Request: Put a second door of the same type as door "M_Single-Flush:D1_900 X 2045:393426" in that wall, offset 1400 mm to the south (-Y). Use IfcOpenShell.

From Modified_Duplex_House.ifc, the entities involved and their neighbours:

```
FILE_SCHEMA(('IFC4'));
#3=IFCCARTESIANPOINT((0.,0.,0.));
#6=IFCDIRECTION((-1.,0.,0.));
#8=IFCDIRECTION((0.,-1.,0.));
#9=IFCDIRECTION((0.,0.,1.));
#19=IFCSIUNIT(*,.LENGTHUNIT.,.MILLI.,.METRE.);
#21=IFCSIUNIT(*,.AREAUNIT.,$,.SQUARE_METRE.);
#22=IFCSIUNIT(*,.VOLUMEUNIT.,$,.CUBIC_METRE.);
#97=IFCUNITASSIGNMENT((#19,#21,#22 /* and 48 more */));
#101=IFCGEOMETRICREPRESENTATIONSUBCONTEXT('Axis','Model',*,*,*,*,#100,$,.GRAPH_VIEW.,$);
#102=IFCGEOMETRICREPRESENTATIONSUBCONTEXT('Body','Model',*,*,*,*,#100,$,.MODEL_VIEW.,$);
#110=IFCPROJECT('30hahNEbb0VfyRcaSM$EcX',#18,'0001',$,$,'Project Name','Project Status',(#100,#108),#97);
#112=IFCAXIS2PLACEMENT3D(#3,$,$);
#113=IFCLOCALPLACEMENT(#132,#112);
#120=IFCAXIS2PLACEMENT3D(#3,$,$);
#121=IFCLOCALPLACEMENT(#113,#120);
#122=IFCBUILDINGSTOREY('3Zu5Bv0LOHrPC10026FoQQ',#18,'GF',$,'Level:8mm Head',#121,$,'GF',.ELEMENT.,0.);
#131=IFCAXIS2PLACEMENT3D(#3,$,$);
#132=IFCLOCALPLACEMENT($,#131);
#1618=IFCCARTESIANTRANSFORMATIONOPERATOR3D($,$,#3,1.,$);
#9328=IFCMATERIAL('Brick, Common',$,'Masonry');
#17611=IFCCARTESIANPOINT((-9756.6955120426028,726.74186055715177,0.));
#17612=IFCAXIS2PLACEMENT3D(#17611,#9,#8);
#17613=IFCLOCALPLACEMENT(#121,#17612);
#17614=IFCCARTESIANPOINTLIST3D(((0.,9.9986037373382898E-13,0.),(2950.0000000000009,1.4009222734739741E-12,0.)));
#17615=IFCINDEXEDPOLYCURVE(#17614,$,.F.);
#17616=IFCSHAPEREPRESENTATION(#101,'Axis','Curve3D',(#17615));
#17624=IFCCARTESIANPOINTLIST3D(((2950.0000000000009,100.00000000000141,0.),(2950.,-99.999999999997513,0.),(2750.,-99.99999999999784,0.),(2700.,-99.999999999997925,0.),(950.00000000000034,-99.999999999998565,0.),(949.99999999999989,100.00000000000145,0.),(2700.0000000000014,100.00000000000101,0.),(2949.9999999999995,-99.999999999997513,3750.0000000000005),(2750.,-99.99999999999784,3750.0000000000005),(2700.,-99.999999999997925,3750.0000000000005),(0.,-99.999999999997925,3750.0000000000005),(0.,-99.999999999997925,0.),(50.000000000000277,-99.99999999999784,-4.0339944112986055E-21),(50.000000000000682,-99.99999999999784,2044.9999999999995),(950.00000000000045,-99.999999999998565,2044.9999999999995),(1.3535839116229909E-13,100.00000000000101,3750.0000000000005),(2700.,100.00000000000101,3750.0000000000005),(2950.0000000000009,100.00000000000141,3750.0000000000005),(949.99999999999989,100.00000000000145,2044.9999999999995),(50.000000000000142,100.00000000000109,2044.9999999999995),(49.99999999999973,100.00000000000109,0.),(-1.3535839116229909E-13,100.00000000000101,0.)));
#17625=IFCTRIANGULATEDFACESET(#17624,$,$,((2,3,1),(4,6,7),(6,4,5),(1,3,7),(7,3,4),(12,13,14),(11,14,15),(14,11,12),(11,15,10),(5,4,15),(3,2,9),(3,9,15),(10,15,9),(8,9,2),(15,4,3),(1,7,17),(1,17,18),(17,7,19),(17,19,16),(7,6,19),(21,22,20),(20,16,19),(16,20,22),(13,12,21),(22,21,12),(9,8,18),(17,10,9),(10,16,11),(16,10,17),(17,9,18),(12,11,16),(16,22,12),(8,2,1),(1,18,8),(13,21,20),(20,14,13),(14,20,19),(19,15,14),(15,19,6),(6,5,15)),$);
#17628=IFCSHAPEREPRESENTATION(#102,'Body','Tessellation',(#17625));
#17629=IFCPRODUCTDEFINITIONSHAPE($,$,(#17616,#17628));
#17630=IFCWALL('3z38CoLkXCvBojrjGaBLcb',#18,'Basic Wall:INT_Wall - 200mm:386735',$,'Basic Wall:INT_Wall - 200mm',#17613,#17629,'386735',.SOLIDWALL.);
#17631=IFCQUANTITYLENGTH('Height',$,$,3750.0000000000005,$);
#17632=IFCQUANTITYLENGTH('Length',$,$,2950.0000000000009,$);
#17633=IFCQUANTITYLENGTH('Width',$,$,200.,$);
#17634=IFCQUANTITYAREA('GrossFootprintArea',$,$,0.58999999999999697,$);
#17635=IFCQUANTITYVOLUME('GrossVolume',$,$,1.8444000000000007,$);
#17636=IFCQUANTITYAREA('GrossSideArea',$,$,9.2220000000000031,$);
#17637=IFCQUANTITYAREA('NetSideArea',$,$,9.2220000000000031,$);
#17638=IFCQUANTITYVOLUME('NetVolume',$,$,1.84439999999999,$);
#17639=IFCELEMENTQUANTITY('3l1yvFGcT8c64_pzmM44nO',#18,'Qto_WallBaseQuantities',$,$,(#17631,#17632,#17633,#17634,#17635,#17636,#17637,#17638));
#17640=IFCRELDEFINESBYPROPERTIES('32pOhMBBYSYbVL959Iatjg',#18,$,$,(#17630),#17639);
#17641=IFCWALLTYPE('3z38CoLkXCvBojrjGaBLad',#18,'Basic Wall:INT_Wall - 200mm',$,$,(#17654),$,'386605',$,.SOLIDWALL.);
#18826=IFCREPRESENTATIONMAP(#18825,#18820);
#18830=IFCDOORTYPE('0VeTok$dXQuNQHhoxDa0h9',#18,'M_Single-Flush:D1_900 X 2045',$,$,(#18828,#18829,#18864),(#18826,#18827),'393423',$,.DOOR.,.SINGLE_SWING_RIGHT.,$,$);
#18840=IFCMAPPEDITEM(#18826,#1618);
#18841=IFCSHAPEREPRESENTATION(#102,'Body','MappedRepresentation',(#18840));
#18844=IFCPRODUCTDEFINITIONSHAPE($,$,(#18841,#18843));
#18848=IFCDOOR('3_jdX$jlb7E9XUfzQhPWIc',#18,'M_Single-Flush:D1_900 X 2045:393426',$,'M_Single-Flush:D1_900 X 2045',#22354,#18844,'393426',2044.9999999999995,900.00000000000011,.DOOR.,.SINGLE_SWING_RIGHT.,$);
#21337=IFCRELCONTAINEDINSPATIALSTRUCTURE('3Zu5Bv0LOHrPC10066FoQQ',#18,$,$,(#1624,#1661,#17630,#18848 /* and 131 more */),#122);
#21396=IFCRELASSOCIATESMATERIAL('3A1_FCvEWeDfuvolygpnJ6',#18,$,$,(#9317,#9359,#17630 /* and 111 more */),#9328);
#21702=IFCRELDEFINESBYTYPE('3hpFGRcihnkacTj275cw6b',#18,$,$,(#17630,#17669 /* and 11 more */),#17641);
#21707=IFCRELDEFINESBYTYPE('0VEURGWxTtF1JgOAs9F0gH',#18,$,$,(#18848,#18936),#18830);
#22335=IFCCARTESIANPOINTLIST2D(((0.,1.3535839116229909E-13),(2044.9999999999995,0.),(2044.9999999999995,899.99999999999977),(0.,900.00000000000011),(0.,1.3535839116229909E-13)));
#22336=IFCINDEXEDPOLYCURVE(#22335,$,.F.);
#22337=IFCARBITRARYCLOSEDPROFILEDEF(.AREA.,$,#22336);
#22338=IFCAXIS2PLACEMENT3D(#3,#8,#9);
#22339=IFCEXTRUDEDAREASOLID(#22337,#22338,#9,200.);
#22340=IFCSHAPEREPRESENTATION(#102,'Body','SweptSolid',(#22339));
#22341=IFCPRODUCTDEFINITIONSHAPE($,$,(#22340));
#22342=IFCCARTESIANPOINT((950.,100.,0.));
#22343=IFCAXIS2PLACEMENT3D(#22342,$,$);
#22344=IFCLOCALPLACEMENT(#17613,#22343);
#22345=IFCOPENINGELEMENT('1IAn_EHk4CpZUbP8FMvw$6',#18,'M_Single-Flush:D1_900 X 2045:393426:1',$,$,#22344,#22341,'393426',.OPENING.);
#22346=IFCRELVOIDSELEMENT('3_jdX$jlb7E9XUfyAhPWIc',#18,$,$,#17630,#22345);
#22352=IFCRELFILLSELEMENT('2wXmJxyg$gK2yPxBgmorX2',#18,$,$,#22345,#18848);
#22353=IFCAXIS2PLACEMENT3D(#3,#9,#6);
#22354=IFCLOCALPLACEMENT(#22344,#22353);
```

```python
import ifcopenshell
import ifcopenshell.api.feature
import ifcopenshell.api.geometry
import ifcopenshell.api.pset
import ifcopenshell.api.root
import ifcopenshell.geom
import ifcopenshell.util.element
import ifcopenshell.util.placement
import ifcopenshell.util.shape
import ifcopenshell.util.unit

model = ifcopenshell.open("Modified_Duplex_House.ifc")
area_scale = ifcopenshell.util.unit.calculate_unit_scale(model, "AREAUNIT")
volume_scale = ifcopenshell.util.unit.calculate_unit_scale(model, "VOLUMEUNIT")
settings = ifcopenshell.geom.settings()


def volume(element):
    """Net volume in cubic metres, openings subtracted."""
    shape = ifcopenshell.geom.create_shape(settings, element)
    return ifcopenshell.util.shape.get_volume(shape.geometry)


def reuse_history(source, copy):
    """copy_class also copies each property set's owner history, people and application; keep the originals."""
    for rel in copy.IsDefinedBy:
        if rel.is_a("IfcRelDefinesByProperties") and (history := rel.RelatingPropertyDefinition.OwnerHistory):
            rel.RelatingPropertyDefinition.OwnerHistory = source.OwnerHistory
            ifcopenshell.util.element.remove_deep2(model, history)


door = model.by_id(18848)
opening = door.FillsVoids[0].RelatingOpeningElement
wall = opening.VoidsElements[0].RelatingBuildingElement
before = volume(wall)
shift = ifcopenshell.util.placement.get_local_placement(wall.ObjectPlacement)[:3, 0] * 1400.0

# copy_class copies the void relationship, type, container and properties, but no geometry.
new_opening = ifcopenshell.api.root.copy_class(model, product=opening)
new_opening.Representation = ifcopenshell.util.element.copy_deep(
    model, opening.Representation, exclude=["IfcGeometricRepresentationContext", "IfcRepresentationMap"]
)
new_opening.Name = "M_Single-Flush:D1_900 X 2045"
new_opening.Tag = None
reuse_history(opening, new_opening)
new_door = ifcopenshell.api.root.copy_class(model, product=door)
new_door.Representation = ifcopenshell.util.element.copy_deep(
    model, door.Representation, exclude=["IfcGeometricRepresentationContext", "IfcRepresentationMap"]
)
new_door.Name = "M_Single-Flush:D1_900 X 2045"
new_door.Tag = None
reuse_history(door, new_door)
ifcopenshell.api.feature.add_filling(model, opening=new_opening, element=new_door)

for old, new in ((opening, new_opening), (door, new_door)):
    matrix = ifcopenshell.util.placement.get_local_placement(old.ObjectPlacement)
    matrix[:3, 3] += shift
    ifcopenshell.api.geometry.edit_object_placement(model, product=new, matrix=matrix, is_si=False)

after = volume(wall)
thickness = 0.2  # wall thickness in metres

# Update the wall's stored quantities.
qto = model.by_id(ifcopenshell.util.element.get_pset(wall, "Qto_WallBaseQuantities", should_inherit=False)["id"])
ifcopenshell.api.pset.edit_qto(model, qto=qto, properties={
    "NetSideArea": after / thickness / area_scale,
    "NetVolume": after / volume_scale,
})

print(f"wall volume {before:.3f} -> {after:.3f} m3")

model.write("Modified_Duplex_House_v2.ifc")
```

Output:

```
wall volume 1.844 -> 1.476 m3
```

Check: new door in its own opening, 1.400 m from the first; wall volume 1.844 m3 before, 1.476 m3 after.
